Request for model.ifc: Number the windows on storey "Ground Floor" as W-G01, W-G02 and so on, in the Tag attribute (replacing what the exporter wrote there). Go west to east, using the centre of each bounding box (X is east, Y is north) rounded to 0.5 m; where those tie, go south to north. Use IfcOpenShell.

First a look at what the model holds.

```python
import ifcopenshell
import ifcopenshell.util.element
import ifcopenshell.util.placement

model = ifcopenshell.open("model.ifc")
print(model.schema)
storey = next(s for s in model.by_type("IfcBuildingStorey") if s.Name == "Ground Floor")
windows = [e for e in ifcopenshell.util.element.get_decomposition(storey) if e.is_a("IfcWindow")]
for e in sorted(windows, key=lambda e: e.id()):
    origin = ifcopenshell.util.placement.get_local_placement(e.ObjectPlacement)[:3, 3]
    print(e.id(), e.Tag, e.Name, origin.round(2) + 0.0, sep=" | ")
```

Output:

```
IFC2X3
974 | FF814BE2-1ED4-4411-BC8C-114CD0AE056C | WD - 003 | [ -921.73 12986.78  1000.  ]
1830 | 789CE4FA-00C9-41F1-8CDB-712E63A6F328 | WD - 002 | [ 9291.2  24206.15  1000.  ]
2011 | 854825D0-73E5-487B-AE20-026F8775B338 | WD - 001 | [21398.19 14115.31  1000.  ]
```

```python
import ifcopenshell
import ifcopenshell.geom
import ifcopenshell.util.element
import ifcopenshell.util.shape

model = ifcopenshell.open("model.ifc")
settings = ifcopenshell.geom.settings()
settings.set("use-world-coords", True)


def centre(element):
    shape = ifcopenshell.geom.create_shape(settings, element)
    return ifcopenshell.util.shape.get_bbox_centroid(shape.geometry)


storey = next(s for s in model.by_type("IfcBuildingStorey") if s.Name == "Ground Floor")
windows = [e for e in ifcopenshell.util.element.get_decomposition(storey) if e.is_a("IfcWindow")]

# Insertion points can sit at a corner or the storey origin, so sort by the geometry (in metres).
centres = {e: centre(e) for e in windows}
windows.sort(key=lambda e: (round(centres[e][0] / 0.5), centres[e][1]))

for i, e in enumerate(windows, start=1):
    number = f"W-G{i:02d}"
    e.Tag = number
    print(e.id(), number)

model.write("model_updated.ifc")
```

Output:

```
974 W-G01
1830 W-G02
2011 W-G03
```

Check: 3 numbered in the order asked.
